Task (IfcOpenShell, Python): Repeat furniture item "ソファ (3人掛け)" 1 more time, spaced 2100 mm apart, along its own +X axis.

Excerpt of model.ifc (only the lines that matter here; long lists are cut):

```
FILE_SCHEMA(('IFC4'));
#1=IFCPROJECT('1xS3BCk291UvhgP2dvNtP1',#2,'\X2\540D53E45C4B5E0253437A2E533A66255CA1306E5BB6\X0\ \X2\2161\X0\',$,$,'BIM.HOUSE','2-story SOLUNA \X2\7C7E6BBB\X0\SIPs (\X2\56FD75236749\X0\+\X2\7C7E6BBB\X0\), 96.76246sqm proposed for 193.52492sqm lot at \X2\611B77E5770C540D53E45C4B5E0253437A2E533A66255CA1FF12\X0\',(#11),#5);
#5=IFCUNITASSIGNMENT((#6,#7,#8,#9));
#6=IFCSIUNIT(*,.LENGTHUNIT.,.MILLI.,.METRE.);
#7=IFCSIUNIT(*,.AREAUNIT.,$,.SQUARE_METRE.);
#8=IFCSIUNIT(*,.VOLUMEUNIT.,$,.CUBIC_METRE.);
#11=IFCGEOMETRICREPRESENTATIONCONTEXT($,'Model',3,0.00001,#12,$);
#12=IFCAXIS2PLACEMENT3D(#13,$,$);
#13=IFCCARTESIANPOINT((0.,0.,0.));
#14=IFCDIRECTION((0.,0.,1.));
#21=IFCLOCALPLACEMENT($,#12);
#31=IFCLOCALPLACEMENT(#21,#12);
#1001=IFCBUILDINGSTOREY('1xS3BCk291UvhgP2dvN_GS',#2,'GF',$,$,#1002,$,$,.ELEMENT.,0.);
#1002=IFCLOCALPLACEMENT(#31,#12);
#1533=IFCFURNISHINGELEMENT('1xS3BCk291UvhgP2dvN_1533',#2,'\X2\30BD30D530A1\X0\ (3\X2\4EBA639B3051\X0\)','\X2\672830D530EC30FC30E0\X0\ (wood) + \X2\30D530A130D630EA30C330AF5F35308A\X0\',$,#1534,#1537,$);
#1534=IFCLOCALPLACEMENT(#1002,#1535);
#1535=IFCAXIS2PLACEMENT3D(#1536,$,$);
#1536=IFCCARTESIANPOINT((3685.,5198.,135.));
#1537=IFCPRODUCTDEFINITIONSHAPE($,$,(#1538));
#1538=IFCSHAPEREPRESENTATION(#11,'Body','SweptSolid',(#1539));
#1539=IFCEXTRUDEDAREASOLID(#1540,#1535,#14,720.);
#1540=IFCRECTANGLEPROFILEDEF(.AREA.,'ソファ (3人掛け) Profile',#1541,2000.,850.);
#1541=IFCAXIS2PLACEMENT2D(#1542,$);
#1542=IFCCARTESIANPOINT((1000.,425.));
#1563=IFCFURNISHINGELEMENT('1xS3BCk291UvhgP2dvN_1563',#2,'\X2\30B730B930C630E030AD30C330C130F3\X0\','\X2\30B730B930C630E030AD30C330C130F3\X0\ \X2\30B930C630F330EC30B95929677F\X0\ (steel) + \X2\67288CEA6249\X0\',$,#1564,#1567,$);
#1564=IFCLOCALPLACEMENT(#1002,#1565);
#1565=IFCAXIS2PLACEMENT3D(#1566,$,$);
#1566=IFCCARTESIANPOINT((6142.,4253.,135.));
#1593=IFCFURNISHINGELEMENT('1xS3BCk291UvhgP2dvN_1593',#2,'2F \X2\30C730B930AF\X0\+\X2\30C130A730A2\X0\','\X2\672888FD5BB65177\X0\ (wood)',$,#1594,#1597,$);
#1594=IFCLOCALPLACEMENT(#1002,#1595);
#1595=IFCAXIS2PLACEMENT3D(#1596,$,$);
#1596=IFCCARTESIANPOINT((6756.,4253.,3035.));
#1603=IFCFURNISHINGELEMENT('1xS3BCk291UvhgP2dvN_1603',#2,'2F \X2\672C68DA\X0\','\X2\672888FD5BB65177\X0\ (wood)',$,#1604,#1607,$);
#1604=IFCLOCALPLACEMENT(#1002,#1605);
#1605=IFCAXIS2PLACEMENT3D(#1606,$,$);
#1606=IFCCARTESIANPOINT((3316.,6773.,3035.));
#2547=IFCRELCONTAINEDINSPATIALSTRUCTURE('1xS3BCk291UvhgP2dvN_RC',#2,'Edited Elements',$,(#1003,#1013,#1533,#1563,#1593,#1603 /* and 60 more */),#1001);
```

```python
import ifcopenshell
import ifcopenshell.api.geometry
import ifcopenshell.api.root
import ifcopenshell.util.element
import ifcopenshell.util.placement

model = ifcopenshell.open("model.ifc")


def reuse_history(source, copy):
    """copy_class also copies each property set's owner history, people and application; keep the originals."""
    for rel in copy.IsDefinedBy:
        if rel.is_a("IfcRelDefinesByProperties") and (history := rel.RelatingPropertyDefinition.OwnerHistory):
            rel.RelatingPropertyDefinition.OwnerHistory = source.OwnerHistory
            ifcopenshell.util.element.remove_deep2(model, history)


source = model.by_guid("1xS3BCk291UvhgP2dvN_1533")
base = ifcopenshell.util.placement.get_local_placement(source.ObjectPlacement)
step = base[:3, 0] * 2100.0

for i in range(1, 2):
    copy = ifcopenshell.api.root.copy_class(model, product=source)
    copy.Representation = ifcopenshell.util.element.copy_deep(
        model, source.Representation, exclude=["IfcGeometricRepresentationContext", "IfcRepresentationMap"]
    )
    reuse_history(source, copy)
    matrix = base.copy()
    matrix[:3, 3] += i * step
    print("added at", matrix[:3, 3].round(3) + 0.0)
    ifcopenshell.api.geometry.edit_object_placement(model, product=copy, matrix=matrix, is_si=False)

model.write("model_v2.ifc")
```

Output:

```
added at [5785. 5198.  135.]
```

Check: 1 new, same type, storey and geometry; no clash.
